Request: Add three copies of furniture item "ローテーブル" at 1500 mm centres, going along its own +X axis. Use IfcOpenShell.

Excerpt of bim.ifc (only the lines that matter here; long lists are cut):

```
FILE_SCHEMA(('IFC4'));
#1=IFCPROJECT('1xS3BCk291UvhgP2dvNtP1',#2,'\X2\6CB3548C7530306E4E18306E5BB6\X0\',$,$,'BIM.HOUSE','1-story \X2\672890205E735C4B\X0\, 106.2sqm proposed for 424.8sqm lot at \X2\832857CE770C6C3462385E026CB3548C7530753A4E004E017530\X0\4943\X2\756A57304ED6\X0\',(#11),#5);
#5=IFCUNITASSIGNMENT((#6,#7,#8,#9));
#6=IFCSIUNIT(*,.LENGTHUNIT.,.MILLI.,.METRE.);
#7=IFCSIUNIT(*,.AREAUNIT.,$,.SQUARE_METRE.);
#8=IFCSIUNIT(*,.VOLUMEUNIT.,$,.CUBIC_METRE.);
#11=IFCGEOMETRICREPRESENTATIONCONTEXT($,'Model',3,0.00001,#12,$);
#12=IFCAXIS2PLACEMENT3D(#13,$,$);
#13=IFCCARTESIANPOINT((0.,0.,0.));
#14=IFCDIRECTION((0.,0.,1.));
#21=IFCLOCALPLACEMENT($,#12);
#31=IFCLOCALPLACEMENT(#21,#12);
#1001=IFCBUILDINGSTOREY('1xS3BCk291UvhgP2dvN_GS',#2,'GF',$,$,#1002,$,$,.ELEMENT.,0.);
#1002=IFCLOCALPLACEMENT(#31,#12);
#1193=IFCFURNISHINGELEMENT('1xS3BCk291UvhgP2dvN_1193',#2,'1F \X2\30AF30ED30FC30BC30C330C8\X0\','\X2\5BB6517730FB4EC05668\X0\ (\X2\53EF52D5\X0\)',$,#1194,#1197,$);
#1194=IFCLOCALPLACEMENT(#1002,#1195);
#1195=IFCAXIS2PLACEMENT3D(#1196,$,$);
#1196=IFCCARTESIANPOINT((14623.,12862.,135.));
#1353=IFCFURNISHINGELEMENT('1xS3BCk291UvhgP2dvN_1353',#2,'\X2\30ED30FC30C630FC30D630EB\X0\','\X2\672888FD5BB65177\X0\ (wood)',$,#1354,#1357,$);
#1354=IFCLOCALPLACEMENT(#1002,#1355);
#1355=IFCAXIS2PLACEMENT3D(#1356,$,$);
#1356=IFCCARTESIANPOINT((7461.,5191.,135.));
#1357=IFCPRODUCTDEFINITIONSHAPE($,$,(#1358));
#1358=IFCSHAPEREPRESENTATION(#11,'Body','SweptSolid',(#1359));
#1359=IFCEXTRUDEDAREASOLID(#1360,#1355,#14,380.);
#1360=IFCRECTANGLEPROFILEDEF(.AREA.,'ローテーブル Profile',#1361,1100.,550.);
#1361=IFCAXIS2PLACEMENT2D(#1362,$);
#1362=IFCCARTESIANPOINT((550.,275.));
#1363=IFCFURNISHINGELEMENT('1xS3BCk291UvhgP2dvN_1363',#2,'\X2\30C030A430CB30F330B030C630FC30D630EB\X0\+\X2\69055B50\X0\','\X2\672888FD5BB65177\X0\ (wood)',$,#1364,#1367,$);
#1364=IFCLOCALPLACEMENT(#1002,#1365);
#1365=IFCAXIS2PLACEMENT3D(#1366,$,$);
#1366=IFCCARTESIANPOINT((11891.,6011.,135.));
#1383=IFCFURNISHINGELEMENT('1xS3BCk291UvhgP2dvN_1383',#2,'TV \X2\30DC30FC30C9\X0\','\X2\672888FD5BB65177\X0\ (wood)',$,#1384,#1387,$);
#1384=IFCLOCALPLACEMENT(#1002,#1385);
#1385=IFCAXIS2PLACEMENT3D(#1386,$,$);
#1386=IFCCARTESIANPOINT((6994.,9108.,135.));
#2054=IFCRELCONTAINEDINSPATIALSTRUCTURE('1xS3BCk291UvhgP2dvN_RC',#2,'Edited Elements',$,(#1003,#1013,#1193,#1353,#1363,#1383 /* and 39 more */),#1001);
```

```python
import ifcopenshell
import ifcopenshell.api.geometry
import ifcopenshell.api.root
import ifcopenshell.util.element
import ifcopenshell.util.placement

model = ifcopenshell.open("bim.ifc")


def reuse_history(source, copy):
    """copy_class also copies each property set's owner history, people and application; keep the originals."""
    for rel in copy.IsDefinedBy:
        if rel.is_a("IfcRelDefinesByProperties") and (history := rel.RelatingPropertyDefinition.OwnerHistory):
            rel.RelatingPropertyDefinition.OwnerHistory = source.OwnerHistory
            ifcopenshell.util.element.remove_deep2(model, history)


source = model.by_guid("1xS3BCk291UvhgP2dvN_1353")
base = ifcopenshell.util.placement.get_local_placement(source.ObjectPlacement)
step = base[:3, 0] * 1500.0

for i in range(1, 4):
    copy = ifcopenshell.api.root.copy_class(model, product=source)
    copy.Representation = ifcopenshell.util.element.copy_deep(
        model, source.Representation, exclude=["IfcGeometricRepresentationContext", "IfcRepresentationMap"]
    )
    reuse_history(source, copy)
    matrix = base.copy()
    matrix[:3, 3] += i * step
    print("added at", matrix[:3, 3].round(3) + 0.0)
    ifcopenshell.api.geometry.edit_object_placement(model, product=copy, matrix=matrix, is_si=False)

model.write("bim-out.ifc")
```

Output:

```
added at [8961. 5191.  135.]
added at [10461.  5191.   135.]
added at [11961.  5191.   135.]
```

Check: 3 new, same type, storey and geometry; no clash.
